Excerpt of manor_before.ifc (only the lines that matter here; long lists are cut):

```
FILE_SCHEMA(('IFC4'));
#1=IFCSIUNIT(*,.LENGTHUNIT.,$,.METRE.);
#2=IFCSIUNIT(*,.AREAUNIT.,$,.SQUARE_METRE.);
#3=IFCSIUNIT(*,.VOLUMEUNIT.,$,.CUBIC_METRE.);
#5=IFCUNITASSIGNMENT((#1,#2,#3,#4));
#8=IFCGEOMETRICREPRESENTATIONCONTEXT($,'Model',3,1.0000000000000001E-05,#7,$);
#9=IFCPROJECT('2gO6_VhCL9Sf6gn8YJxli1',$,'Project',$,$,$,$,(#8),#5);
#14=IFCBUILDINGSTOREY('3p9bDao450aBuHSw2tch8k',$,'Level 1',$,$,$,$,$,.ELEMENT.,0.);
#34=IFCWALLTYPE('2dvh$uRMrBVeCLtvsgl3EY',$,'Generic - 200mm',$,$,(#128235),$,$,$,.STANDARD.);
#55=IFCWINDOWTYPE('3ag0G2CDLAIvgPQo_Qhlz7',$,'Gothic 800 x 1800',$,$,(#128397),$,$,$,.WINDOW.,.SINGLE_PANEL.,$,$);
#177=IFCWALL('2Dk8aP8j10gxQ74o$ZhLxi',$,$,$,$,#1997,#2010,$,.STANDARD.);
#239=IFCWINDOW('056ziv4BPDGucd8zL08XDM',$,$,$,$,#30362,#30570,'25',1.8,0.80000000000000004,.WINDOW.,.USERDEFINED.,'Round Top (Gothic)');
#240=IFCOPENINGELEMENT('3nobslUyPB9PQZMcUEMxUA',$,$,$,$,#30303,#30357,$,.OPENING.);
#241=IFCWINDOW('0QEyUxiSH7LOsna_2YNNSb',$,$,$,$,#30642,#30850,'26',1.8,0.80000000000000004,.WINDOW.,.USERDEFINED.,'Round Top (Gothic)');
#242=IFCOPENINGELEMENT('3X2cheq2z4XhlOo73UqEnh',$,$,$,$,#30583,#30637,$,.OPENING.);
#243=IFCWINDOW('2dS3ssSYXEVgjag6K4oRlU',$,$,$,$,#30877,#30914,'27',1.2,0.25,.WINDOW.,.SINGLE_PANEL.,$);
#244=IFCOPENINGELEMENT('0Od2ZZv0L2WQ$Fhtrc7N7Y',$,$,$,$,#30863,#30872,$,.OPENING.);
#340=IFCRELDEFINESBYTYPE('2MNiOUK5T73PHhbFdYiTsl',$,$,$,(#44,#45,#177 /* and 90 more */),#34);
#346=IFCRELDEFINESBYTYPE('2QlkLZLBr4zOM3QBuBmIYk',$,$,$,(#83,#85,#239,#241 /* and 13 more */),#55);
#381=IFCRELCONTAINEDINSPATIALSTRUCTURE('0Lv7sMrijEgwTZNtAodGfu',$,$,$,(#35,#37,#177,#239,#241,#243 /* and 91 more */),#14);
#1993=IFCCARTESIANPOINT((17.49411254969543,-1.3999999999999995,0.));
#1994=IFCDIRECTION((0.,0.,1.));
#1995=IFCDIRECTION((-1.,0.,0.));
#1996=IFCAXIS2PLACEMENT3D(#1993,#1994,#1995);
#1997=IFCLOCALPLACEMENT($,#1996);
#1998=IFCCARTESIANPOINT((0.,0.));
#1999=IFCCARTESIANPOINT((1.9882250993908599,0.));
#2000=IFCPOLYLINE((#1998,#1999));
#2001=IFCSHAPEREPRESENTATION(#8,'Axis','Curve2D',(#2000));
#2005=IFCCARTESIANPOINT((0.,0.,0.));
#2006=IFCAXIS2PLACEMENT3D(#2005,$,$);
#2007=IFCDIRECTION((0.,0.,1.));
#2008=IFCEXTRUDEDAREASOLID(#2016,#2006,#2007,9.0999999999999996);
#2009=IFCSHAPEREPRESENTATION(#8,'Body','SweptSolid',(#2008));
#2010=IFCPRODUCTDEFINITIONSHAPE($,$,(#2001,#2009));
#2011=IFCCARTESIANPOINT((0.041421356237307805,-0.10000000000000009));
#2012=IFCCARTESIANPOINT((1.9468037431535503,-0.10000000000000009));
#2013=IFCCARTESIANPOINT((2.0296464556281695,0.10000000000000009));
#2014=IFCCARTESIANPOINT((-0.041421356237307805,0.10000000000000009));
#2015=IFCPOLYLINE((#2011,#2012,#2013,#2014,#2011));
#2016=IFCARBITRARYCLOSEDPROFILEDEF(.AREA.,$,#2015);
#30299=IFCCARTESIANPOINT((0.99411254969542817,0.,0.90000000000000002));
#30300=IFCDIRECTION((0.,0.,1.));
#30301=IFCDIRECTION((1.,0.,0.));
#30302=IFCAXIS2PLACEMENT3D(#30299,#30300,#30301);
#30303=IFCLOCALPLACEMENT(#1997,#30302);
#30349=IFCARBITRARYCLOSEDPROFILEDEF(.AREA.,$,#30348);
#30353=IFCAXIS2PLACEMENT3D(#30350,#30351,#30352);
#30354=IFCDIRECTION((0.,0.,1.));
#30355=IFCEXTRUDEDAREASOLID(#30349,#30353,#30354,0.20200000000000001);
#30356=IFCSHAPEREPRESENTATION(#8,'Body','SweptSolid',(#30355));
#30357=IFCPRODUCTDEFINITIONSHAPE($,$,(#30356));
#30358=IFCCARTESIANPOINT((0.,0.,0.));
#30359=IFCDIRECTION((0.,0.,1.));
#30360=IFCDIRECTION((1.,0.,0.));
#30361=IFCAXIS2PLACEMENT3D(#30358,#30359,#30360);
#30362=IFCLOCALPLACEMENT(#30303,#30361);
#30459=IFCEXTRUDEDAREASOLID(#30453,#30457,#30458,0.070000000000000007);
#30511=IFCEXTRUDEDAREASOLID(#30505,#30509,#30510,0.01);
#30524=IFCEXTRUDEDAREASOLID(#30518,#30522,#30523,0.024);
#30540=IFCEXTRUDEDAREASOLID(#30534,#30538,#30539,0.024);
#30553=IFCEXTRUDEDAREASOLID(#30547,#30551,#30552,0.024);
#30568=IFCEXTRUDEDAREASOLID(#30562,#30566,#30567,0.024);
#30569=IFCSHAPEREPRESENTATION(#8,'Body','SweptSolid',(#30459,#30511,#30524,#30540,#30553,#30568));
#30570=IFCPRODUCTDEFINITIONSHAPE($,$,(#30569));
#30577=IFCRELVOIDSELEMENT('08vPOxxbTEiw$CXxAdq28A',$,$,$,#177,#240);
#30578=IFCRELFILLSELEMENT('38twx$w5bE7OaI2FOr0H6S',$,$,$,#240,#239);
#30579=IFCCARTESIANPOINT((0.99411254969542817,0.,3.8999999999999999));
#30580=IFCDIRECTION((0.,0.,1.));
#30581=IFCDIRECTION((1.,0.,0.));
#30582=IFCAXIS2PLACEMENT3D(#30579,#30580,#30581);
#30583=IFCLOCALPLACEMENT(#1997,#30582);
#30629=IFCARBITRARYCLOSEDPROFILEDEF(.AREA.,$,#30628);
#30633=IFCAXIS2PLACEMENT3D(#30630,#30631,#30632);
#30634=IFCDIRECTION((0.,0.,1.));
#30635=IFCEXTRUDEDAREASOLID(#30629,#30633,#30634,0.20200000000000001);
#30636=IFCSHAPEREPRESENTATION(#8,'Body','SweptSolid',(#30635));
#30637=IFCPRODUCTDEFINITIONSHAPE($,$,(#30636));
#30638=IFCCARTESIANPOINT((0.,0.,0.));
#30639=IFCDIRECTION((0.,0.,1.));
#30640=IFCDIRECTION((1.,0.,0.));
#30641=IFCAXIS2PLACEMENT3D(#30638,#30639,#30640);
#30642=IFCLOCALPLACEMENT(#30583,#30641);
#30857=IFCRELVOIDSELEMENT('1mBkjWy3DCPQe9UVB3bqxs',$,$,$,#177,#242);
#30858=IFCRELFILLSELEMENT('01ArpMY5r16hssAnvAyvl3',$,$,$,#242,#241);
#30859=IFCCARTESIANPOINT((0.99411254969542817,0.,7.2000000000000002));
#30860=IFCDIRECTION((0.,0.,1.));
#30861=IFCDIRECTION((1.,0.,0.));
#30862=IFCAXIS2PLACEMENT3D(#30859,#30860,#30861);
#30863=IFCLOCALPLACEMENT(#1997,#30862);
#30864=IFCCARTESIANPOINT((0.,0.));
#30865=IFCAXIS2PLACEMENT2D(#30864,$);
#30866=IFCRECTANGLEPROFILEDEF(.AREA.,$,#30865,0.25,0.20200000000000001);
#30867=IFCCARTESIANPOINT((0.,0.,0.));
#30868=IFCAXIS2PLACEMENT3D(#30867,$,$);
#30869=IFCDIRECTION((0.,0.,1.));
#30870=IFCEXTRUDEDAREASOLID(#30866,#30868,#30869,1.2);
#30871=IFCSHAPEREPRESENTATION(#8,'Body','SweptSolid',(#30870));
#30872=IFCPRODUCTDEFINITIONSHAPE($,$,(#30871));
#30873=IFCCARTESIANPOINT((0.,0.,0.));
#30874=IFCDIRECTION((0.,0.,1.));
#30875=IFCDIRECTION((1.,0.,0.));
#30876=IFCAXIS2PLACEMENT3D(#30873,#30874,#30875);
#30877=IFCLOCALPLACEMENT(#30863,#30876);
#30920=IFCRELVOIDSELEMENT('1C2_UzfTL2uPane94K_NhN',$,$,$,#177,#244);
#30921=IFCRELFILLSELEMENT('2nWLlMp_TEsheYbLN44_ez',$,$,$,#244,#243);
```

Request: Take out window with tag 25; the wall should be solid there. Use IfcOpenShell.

```python
import ifcopenshell
import ifcopenshell.api.feature
import ifcopenshell.api.root
import ifcopenshell.geom
import ifcopenshell.util.shape

model = ifcopenshell.open("manor_before.ifc")
settings = ifcopenshell.geom.settings()


def volume(element):
    """Net volume in cubic metres, openings subtracted."""
    shape = ifcopenshell.geom.create_shape(settings, element)
    return ifcopenshell.util.shape.get_volume(shape.geometry)


window = model.by_guid("056ziv4BPDGucd8zL08XDM")
opening = window.FillsVoids[0].RelatingOpeningElement
wall = opening.VoidsElements[0].RelatingBuildingElement
before = volume(wall)

ifcopenshell.api.root.remove_product(model, product=window)
ifcopenshell.api.feature.remove_feature(model, feature=opening)

after = volume(wall)

print(f"wall volume {before:.3f} -> {after:.3f} m3")

model.write("manor_before_rev.ifc")
```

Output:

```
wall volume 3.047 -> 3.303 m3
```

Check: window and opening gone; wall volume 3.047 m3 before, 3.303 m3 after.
